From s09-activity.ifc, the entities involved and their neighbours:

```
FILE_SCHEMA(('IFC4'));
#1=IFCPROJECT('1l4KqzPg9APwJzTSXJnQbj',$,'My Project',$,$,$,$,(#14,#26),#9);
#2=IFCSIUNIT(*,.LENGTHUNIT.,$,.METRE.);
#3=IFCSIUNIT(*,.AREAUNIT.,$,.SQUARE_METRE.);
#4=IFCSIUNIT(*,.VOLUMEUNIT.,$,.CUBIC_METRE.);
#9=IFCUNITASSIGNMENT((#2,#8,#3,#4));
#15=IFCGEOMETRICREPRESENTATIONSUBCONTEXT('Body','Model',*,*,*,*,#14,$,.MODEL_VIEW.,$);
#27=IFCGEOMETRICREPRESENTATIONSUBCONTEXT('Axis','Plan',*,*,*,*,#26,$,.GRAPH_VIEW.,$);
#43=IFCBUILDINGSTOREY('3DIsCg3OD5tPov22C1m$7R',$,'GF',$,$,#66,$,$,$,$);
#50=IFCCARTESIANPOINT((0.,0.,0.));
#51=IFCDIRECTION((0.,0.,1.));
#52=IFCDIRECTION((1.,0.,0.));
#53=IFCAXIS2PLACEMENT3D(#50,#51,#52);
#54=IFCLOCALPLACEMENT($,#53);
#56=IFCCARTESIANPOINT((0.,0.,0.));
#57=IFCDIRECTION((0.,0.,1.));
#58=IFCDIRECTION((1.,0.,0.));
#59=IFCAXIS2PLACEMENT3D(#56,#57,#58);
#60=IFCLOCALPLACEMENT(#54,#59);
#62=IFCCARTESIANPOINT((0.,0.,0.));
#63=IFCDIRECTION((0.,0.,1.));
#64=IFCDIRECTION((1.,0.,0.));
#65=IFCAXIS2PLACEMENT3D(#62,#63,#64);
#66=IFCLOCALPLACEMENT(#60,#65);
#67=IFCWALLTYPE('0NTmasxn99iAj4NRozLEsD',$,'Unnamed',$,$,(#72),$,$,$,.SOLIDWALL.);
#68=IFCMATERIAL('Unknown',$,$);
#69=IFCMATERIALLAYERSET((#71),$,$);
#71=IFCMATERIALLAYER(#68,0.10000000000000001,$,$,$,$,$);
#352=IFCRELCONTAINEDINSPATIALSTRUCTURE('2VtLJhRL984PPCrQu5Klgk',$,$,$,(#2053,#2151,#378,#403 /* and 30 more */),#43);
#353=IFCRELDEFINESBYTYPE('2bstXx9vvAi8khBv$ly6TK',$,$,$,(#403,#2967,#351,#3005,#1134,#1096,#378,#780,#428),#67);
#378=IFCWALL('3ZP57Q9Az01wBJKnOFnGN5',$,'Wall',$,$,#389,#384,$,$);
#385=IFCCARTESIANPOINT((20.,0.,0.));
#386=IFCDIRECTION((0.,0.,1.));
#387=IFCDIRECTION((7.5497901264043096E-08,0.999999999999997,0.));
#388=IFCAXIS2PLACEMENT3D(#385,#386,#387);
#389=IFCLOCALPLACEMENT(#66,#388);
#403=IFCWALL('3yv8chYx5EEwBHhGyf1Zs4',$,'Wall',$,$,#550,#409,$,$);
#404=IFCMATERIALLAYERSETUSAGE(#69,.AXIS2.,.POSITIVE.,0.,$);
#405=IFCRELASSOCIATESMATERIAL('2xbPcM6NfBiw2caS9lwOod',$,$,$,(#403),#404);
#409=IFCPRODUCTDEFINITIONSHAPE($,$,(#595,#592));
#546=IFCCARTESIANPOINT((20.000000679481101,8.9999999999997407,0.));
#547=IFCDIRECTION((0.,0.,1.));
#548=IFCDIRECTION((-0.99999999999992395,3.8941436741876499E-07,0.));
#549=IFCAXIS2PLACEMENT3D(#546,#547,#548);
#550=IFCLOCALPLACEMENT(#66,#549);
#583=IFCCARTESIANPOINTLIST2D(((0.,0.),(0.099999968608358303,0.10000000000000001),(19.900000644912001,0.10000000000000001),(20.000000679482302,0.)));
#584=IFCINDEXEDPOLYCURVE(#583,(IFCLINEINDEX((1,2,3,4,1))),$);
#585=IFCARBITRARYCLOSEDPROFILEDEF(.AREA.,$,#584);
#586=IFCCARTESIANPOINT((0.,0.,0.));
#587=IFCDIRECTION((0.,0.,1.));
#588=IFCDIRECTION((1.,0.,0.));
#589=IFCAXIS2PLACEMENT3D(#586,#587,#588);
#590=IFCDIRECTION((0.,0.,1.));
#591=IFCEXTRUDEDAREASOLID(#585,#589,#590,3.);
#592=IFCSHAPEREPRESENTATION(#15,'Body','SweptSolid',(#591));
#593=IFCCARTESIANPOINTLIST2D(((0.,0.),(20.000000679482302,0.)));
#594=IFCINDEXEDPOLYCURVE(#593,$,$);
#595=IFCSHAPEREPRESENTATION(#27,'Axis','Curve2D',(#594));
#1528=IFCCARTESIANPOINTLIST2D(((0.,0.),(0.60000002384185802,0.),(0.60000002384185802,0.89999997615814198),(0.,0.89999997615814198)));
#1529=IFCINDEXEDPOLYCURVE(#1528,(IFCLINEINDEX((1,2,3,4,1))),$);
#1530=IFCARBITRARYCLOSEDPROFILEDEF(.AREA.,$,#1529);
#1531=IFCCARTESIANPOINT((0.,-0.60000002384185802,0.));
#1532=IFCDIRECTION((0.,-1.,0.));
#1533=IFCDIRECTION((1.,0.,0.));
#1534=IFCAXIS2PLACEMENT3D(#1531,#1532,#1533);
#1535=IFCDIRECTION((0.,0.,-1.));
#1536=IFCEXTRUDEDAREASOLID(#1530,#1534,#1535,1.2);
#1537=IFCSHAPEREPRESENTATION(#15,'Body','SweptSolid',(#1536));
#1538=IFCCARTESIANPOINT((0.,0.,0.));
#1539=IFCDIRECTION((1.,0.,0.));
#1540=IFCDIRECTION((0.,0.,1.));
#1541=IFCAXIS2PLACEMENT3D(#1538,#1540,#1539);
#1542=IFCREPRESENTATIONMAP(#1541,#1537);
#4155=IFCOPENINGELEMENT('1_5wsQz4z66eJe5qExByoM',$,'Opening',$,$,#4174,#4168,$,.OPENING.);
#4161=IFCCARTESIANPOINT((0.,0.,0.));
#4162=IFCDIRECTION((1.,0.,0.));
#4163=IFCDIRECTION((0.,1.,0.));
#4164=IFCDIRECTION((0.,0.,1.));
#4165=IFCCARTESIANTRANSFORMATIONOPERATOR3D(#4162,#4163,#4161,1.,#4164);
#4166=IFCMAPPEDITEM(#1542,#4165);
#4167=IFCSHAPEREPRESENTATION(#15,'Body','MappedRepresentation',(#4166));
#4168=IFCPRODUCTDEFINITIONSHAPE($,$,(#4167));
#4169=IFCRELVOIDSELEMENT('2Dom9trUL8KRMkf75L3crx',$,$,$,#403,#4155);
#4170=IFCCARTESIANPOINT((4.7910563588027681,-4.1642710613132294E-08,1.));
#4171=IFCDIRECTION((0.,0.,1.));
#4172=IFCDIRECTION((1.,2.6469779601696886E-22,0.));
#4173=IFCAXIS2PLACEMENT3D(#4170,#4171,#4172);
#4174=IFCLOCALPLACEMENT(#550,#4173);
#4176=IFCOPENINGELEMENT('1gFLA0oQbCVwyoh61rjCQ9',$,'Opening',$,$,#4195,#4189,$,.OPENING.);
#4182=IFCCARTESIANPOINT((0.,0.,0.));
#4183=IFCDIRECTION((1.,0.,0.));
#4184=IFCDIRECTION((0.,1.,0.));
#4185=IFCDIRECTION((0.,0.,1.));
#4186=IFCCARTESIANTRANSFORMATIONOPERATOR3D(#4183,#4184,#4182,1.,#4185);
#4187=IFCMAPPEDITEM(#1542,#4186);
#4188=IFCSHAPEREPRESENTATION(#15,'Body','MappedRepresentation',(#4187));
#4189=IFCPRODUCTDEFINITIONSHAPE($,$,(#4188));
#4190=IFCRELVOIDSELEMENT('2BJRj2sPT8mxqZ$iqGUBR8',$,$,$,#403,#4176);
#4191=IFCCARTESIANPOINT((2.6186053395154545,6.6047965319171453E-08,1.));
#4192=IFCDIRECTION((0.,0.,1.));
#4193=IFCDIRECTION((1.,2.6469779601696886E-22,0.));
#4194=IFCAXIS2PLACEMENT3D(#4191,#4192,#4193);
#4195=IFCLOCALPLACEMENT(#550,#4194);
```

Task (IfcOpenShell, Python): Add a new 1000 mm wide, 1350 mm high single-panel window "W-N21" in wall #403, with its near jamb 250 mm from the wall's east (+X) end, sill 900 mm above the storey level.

```python
import numpy as np
import ifcopenshell
import ifcopenshell.api.feature
import ifcopenshell.api.geometry
import ifcopenshell.api.root
import ifcopenshell.api.spatial
import ifcopenshell.geom
import ifcopenshell.util.element
import ifcopenshell.util.placement
import ifcopenshell.util.representation
import ifcopenshell.util.shape
import ifcopenshell.util.unit

model = ifcopenshell.open("s09-activity.ifc")
unit_scale = ifcopenshell.util.unit.calculate_unit_scale(model)
settings = ifcopenshell.geom.settings()


def volume(element):
    """Net volume in cubic metres, openings subtracted."""
    shape = ifcopenshell.geom.create_shape(settings, element)
    return ifcopenshell.util.shape.get_volume(shape.geometry)


wall = model.by_guid("3yv8chYx5EEwBHhGyf1Zs4")
storey = ifcopenshell.util.element.get_container(wall, ifc_class="IfcBuildingStorey")
context = ifcopenshell.util.representation.get_context(model, "Model", "Body", "MODEL_VIEW")
before = volume(wall)

width, height, from_end, sill = 1, 1.35, 0.25, 0.9  # metres

# The wall runs along its own X axis, and the end named is its -X end.
wall_shape = ifcopenshell.geom.create_shape(settings, wall)
x, y, z = ifcopenshell.util.shape.get_vertices(wall_shape.geometry).T
start = x.min() + from_end
face, thickness = float(y.min()), float(y.max() - y.min())
wall_matrix = ifcopenshell.util.placement.get_local_placement(wall.ObjectPlacement)
level = ifcopenshell.util.placement.get_local_placement(storey.ObjectPlacement)[2, 3]


def in_wall(x, y):
    """Placement at x, y metres in the wall's axes, at sill height."""
    matrix = wall_matrix.copy()
    matrix[:, 3] = wall_matrix @ np.array([x / unit_scale, y / unit_scale, 0.0, 1.0])
    matrix[2, 3] = level + sill / unit_scale
    return matrix


# Opening: a box that overshoots both wall faces by 50 mm.
opening = ifcopenshell.api.root.create_entity(model, ifc_class="IfcOpeningElement", predefined_type="OPENING")
box = ifcopenshell.api.geometry.add_wall_representation(
    model, context=context, length=width, height=height, thickness=thickness + 0.1
)
ifcopenshell.api.geometry.assign_representation(model, product=opening, representation=box)
ifcopenshell.api.geometry.edit_object_placement(model, product=opening, matrix=in_wall(start, face - 0.05), is_si=False)
ifcopenshell.api.feature.add_feature(model, feature=opening, element=wall)

window = ifcopenshell.api.root.create_entity(model, ifc_class="IfcWindow", name="W-N21", predefined_type="WINDOW")
window.OverallWidth, window.OverallHeight = width / unit_scale, height / unit_scale
window.PartitioningType = "SINGLE_PANEL"
body = ifcopenshell.api.geometry.add_window_representation(
    model,
    context=context,
    overall_width=window.OverallWidth,
    overall_height=window.OverallHeight,
    partition_type="SINGLE_PANEL",
)
ifcopenshell.api.geometry.assign_representation(model, product=window, representation=body)
ifcopenshell.api.spatial.assign_container(model, products=[window], relating_structure=storey)
ifcopenshell.api.feature.add_filling(model, opening=opening, element=window)

# Centre the window in the wall's thickness.
ifcopenshell.api.geometry.edit_object_placement(model, product=window, matrix=in_wall(start, face), is_si=False)
window_shape = ifcopenshell.geom.create_shape(settings, window)
depth = ifcopenshell.util.shape.get_vertices(window_shape.geometry)[:, 1]
offset = face + thickness / 2 - (depth.min() + depth.max()) / 2
ifcopenshell.api.geometry.edit_object_placement(model, product=window, matrix=in_wall(start, offset), is_si=False)

after = volume(wall)

print(f"wall volume {before:.3f} -> {after:.3f} m3")

model.write("s09-activity_rev.ifc")
```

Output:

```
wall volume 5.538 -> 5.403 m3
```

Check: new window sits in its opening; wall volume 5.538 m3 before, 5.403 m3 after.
